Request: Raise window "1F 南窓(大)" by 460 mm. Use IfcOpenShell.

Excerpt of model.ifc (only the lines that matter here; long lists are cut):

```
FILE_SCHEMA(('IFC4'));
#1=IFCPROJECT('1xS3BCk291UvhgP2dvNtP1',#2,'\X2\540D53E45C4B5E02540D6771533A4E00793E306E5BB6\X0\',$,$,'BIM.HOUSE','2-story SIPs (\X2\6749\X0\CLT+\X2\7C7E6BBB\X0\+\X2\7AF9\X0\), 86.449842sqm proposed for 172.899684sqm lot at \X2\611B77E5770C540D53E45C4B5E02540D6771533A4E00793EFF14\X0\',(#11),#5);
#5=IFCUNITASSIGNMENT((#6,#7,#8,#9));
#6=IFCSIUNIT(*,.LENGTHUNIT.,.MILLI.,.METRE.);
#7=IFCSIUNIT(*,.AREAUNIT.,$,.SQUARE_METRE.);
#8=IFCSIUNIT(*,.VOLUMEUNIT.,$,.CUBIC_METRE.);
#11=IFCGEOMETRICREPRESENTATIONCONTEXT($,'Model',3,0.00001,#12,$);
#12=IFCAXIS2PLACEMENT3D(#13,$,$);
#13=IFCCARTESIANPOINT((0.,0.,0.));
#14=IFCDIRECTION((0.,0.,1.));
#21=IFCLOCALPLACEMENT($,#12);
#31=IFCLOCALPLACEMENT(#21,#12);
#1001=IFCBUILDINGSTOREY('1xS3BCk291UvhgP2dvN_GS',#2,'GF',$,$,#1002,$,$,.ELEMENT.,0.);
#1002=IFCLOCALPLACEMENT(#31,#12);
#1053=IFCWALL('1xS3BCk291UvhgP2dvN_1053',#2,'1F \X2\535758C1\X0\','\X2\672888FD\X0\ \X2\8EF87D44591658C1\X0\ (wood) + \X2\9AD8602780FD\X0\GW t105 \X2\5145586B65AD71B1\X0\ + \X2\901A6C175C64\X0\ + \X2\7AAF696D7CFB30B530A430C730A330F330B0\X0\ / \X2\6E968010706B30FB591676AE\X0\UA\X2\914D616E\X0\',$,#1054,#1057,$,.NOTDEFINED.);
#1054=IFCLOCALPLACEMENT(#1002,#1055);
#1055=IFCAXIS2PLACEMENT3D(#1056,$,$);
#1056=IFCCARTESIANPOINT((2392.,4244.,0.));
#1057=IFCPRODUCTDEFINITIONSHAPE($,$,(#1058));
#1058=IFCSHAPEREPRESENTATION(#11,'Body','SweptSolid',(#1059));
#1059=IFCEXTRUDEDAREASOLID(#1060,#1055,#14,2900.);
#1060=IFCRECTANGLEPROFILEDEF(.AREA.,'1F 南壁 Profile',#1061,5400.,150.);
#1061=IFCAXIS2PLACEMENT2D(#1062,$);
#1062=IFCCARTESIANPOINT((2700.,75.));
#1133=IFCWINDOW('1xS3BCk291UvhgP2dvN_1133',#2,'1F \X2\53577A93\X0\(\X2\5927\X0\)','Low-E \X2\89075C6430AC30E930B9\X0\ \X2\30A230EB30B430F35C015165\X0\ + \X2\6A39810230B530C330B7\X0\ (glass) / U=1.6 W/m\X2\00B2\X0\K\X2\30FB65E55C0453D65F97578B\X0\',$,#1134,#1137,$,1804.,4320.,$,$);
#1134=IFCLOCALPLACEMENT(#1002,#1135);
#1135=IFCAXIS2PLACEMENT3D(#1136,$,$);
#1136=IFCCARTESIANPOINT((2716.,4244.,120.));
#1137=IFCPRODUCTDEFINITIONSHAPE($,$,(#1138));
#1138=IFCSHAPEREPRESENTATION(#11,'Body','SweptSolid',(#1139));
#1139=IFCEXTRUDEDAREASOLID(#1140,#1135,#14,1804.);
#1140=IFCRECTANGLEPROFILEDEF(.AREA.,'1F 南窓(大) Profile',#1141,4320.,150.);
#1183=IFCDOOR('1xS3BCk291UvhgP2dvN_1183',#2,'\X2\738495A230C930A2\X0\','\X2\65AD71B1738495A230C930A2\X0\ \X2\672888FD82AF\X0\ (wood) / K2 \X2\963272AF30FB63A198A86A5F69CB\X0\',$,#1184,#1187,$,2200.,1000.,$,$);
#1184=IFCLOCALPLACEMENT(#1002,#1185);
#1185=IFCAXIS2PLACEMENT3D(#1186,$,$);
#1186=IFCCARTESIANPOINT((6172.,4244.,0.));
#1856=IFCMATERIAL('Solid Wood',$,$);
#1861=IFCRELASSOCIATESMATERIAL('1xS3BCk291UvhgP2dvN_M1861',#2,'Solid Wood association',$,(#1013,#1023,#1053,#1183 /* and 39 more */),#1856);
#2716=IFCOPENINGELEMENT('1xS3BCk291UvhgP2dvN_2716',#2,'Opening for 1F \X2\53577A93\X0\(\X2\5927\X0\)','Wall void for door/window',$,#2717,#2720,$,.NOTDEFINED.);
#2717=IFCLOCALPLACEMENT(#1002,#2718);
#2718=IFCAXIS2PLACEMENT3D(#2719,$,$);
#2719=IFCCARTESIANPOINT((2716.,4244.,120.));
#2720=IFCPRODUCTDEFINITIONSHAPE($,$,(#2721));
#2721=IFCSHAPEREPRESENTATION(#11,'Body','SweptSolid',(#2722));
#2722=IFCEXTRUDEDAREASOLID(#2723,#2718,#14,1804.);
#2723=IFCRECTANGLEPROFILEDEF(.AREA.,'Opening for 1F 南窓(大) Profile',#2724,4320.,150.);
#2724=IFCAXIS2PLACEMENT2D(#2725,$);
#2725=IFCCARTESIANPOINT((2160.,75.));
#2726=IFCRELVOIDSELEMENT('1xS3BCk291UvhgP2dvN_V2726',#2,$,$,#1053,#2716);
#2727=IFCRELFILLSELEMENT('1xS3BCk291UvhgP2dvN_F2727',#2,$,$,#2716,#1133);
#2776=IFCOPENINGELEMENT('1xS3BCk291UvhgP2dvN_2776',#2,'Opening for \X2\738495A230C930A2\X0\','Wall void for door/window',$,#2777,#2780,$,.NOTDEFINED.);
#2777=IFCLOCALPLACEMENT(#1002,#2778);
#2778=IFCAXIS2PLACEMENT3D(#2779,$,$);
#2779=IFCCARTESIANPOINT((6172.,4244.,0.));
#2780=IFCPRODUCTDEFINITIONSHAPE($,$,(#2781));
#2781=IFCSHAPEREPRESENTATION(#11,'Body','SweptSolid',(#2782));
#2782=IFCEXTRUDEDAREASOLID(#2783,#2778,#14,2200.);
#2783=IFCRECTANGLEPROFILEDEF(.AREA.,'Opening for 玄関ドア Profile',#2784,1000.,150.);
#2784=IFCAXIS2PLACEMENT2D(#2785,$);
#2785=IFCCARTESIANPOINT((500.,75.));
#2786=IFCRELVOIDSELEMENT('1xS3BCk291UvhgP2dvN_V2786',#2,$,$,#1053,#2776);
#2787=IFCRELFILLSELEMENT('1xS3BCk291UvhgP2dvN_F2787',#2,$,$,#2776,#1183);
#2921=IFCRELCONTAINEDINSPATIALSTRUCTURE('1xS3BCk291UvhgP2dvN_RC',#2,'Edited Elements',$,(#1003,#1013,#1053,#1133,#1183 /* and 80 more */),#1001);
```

```python
import numpy as np
import ifcopenshell
import ifcopenshell.api.geometry
import ifcopenshell.util.placement
import ifcopenshell.util.unit

model = ifcopenshell.open("model.ifc")
unit_scale = ifcopenshell.util.unit.calculate_unit_scale(model)

window = model.by_guid("1xS3BCk291UvhgP2dvN_1133")
opening = window.FillsVoids[0].RelatingOpeningElement
dz = 0.46 / unit_scale

shift = np.array([0.0, 0.0, dz])
# The window is not placed relative to its opening, so move both.
for product in (opening, window):
    matrix = ifcopenshell.util.placement.get_local_placement(product.ObjectPlacement)
    matrix[:3, 3] += shift
    ifcopenshell.api.geometry.edit_object_placement(model, product=product, matrix=matrix, is_si=False)

print(f"moved by {dz * unit_scale:+.3f} m")

model.write("model_v2.ifc")
```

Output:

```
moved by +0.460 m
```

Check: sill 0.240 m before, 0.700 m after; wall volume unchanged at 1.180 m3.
